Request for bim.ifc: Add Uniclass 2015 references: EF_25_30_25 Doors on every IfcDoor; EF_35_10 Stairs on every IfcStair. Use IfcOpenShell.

First a look at what the model holds.

```python
import ifcopenshell

model = ifcopenshell.open("bim.ifc")
print(model.schema)
print("classifications:", [c.Name for c in model.by_type("IfcClassification")])
for ifc_class in ("IfcDoor", "IfcRoof", "IfcStair", "IfcWall", "IfcWindow"):
    print(ifc_class, len(model.by_type(ifc_class)))
```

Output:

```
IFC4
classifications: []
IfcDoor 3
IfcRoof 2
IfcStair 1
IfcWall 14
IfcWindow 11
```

```python
import ifcopenshell
import ifcopenshell.api.classification

model = ifcopenshell.open("bim.ifc")

system = ifcopenshell.api.classification.add_classification(model, classification="Uniclass 2015")

codes = {
    "IfcDoor": ("EF_25_30_25", "Doors"),
    "IfcStair": ("EF_35_10", "Stairs"),
}
for ifc_class, (code, name) in codes.items():
    products = model.by_type(ifc_class)
    ifcopenshell.api.classification.add_reference(
        model, products=products, classification=system, identification=code, name=name
    )
    print(code, len(products))

model.write("bim_v2.ifc")
```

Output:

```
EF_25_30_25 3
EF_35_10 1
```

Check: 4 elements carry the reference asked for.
